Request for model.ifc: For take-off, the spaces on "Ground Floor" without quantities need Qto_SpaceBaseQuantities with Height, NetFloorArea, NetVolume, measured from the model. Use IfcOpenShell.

First a look at what the model holds.

```python
import ifcopenshell
import ifcopenshell.util.element
import ifcopenshell.util.unit

model = ifcopenshell.open("model.ifc")
print(model.schema)
for unit_type in ("LENGTHUNIT", "AREAUNIT", "VOLUMEUNIT"):
    print(unit_type, ifcopenshell.util.unit.calculate_unit_scale(model, unit_type))
storey = next(s for s in model.by_type("IfcBuildingStorey") if s.Name == "Ground Floor")
spaces = [e for e in ifcopenshell.util.element.get_decomposition(storey) if e.is_a("IfcSpace")]
for e in sorted(spaces, key=lambda e: e.id()):
    print(e.id(), e.is_a(), e.Name, list(ifcopenshell.util.element.get_psets(e, qtos_only=True)), sep=" | ")
```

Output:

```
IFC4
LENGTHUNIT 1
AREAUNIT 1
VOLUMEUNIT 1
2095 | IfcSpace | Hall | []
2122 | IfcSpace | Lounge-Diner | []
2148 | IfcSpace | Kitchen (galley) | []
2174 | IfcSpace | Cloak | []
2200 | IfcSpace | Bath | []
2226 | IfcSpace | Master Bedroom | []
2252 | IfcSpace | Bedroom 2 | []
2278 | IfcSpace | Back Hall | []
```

```python
import ifcopenshell
import ifcopenshell.api.pset
import ifcopenshell.geom
import ifcopenshell.util.element
import ifcopenshell.util.shape
import ifcopenshell.util.unit

model = ifcopenshell.open("model.ifc")
unit_scale = ifcopenshell.util.unit.calculate_unit_scale(model)
area_scale = ifcopenshell.util.unit.calculate_unit_scale(model, "AREAUNIT")
volume_scale = ifcopenshell.util.unit.calculate_unit_scale(model, "VOLUMEUNIT")
settings = ifcopenshell.geom.settings()

storey = next(s for s in model.by_type("IfcBuildingStorey") if s.Name == "Ground Floor")
spaces = [e for e in ifcopenshell.util.element.get_decomposition(storey) if e.is_a("IfcSpace")]

for e in sorted(spaces, key=lambda e: e.id()):
    if ifcopenshell.util.element.get_psets(e, qtos_only=True, should_inherit=False):
        continue
    # Geometry comes back in metres, in the element's own axes.
    shape = ifcopenshell.geom.create_shape(settings, e)
    values = {
        "Height": ifcopenshell.util.shape.get_z(shape.geometry) / unit_scale,
        "NetFloorArea": ifcopenshell.util.shape.get_footprint_area(shape.geometry) / area_scale,
        "NetVolume": ifcopenshell.util.shape.get_volume(shape.geometry) / volume_scale,
    }
    qto = ifcopenshell.api.pset.add_qto(model, product=e, name="Qto_SpaceBaseQuantities")
    ifcopenshell.api.pset.edit_qto(model, qto=qto, properties=values)
    print(e.id(), {k: round(v, 3) for k, v in values.items()})

model.write("model_updated.ifc")
```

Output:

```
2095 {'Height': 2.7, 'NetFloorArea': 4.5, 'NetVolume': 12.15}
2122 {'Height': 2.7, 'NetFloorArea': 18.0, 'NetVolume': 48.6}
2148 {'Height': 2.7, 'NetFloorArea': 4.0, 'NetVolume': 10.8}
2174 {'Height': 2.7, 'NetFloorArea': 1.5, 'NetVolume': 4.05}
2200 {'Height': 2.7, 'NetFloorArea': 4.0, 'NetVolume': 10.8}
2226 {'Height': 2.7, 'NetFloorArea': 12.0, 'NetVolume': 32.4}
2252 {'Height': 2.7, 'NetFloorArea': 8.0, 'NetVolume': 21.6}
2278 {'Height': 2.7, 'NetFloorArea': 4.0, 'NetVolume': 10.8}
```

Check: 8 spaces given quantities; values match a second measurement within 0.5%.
